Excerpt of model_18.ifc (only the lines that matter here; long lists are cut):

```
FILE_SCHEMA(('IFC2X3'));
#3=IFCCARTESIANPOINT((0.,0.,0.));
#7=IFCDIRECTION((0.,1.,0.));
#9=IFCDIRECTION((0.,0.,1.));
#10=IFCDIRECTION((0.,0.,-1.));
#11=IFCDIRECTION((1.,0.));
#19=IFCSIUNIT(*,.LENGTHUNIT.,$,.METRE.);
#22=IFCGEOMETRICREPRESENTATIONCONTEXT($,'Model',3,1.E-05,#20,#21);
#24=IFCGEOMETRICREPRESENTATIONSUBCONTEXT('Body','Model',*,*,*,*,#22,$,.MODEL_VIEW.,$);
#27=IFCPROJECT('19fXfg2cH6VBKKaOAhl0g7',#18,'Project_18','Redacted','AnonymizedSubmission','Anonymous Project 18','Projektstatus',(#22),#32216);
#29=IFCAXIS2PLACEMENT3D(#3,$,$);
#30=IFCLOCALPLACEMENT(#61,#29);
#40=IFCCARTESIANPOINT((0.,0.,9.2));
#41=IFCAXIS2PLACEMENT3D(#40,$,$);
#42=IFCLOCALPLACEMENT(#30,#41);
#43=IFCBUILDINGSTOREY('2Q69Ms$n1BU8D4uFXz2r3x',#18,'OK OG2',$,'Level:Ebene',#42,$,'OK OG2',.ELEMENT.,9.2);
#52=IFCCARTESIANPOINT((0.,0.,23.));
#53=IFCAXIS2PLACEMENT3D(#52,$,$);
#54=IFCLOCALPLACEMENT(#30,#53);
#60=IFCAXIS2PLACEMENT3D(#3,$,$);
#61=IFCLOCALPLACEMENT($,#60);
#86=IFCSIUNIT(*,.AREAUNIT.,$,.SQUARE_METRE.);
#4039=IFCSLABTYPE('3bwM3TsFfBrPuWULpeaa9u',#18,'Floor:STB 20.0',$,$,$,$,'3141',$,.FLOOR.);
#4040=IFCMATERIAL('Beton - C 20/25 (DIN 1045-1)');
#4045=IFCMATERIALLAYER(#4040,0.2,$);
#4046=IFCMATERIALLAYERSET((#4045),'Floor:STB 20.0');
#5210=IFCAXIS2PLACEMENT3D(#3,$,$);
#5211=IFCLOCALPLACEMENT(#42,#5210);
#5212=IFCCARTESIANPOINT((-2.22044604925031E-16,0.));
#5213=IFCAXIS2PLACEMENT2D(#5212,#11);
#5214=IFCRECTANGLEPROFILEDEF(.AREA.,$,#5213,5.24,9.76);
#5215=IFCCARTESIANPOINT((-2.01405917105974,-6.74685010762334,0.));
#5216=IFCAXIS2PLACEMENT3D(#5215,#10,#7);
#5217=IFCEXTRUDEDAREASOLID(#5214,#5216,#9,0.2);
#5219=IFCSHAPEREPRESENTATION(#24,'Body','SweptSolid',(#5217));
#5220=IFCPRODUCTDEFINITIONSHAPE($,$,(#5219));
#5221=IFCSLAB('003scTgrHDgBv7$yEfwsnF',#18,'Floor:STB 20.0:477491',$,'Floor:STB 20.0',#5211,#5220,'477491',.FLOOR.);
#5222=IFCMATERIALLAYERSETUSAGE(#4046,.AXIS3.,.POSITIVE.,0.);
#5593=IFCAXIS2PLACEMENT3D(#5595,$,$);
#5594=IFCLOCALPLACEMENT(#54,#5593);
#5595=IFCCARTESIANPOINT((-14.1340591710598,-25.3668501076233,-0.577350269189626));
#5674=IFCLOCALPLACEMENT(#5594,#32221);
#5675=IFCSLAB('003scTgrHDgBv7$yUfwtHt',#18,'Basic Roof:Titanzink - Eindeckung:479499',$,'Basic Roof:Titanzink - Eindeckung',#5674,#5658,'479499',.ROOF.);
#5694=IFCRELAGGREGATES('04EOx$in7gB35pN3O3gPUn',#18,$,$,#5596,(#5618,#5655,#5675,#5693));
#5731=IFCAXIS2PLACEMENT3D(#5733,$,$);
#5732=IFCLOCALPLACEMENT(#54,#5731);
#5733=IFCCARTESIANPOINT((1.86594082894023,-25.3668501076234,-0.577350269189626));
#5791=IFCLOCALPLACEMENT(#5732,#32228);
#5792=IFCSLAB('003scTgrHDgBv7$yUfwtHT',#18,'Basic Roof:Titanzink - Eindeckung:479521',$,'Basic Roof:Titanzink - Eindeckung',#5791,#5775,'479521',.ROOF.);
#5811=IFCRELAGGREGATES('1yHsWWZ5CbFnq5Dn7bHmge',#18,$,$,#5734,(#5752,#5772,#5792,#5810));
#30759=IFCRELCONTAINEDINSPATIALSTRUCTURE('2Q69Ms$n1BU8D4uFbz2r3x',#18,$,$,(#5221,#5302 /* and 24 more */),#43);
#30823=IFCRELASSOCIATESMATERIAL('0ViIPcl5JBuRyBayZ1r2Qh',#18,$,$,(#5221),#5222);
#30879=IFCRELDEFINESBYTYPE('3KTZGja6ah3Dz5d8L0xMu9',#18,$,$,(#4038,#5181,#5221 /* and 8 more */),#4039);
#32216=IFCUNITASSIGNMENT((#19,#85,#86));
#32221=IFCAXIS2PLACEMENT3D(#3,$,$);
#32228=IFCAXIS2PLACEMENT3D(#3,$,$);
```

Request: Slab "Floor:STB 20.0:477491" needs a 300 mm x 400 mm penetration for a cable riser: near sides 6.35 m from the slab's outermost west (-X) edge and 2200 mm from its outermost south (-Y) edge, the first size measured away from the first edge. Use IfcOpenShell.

```python
import numpy as np
import ifcopenshell
import ifcopenshell.api.feature
import ifcopenshell.api.geometry
import ifcopenshell.api.root
import ifcopenshell.geom
import ifcopenshell.util.placement
import ifcopenshell.util.representation
import ifcopenshell.util.shape
import ifcopenshell.util.unit

model = ifcopenshell.open("model_18.ifc")
unit_scale = ifcopenshell.util.unit.calculate_unit_scale(model)
settings = ifcopenshell.geom.settings()


def volume(element):
    """Net volume in cubic metres, openings subtracted."""
    shape = ifcopenshell.geom.create_shape(settings, element)
    return ifcopenshell.util.shape.get_volume(shape.geometry)


slab = model.by_id(5221)
before = volume(slab)

# Extent in the slab's own axes, in metres. The edges named are its -X and -Y sides.
slab_shape = ifcopenshell.geom.create_shape(settings, slab)
vertices = ifcopenshell.util.shape.get_vertices(slab_shape.geometry)
x_min, y_min, bottom = vertices.min(axis=0)
top = vertices[:, 2].max()

opening = ifcopenshell.api.root.create_entity(model, ifc_class="IfcOpeningElement", name="Cable riser opening")
context = ifcopenshell.util.representation.get_context(model, "Model", "Body", "MODEL_VIEW")
width, depth = 0.3, 0.4
outline = [(0.0, 0.0), (width, 0.0), (width, depth), (0.0, depth), (0.0, 0.0)]
# Overshoot both faces by 50 mm so the cut is clean.
shape = ifcopenshell.api.geometry.add_slab_representation(
    model, context=context, depth=top - bottom + 0.1, polyline=outline
)
ifcopenshell.api.geometry.assign_representation(model, product=opening, representation=shape)

matrix = ifcopenshell.util.placement.get_local_placement(slab.ObjectPlacement)
matrix[:, 3] = matrix @ np.append(np.array([x_min + 6.35, y_min + 2.2, bottom - 0.05]) / unit_scale, 1.0)
ifcopenshell.api.geometry.edit_object_placement(model, product=opening, matrix=matrix, is_si=False)
ifcopenshell.api.feature.add_feature(model, feature=opening, element=slab)

after = volume(slab)

print(f"slab volume {before:.3f} -> {after:.3f} m3")

model.write("model_18-out.ifc")
```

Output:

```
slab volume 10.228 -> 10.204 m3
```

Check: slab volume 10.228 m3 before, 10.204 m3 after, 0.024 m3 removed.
